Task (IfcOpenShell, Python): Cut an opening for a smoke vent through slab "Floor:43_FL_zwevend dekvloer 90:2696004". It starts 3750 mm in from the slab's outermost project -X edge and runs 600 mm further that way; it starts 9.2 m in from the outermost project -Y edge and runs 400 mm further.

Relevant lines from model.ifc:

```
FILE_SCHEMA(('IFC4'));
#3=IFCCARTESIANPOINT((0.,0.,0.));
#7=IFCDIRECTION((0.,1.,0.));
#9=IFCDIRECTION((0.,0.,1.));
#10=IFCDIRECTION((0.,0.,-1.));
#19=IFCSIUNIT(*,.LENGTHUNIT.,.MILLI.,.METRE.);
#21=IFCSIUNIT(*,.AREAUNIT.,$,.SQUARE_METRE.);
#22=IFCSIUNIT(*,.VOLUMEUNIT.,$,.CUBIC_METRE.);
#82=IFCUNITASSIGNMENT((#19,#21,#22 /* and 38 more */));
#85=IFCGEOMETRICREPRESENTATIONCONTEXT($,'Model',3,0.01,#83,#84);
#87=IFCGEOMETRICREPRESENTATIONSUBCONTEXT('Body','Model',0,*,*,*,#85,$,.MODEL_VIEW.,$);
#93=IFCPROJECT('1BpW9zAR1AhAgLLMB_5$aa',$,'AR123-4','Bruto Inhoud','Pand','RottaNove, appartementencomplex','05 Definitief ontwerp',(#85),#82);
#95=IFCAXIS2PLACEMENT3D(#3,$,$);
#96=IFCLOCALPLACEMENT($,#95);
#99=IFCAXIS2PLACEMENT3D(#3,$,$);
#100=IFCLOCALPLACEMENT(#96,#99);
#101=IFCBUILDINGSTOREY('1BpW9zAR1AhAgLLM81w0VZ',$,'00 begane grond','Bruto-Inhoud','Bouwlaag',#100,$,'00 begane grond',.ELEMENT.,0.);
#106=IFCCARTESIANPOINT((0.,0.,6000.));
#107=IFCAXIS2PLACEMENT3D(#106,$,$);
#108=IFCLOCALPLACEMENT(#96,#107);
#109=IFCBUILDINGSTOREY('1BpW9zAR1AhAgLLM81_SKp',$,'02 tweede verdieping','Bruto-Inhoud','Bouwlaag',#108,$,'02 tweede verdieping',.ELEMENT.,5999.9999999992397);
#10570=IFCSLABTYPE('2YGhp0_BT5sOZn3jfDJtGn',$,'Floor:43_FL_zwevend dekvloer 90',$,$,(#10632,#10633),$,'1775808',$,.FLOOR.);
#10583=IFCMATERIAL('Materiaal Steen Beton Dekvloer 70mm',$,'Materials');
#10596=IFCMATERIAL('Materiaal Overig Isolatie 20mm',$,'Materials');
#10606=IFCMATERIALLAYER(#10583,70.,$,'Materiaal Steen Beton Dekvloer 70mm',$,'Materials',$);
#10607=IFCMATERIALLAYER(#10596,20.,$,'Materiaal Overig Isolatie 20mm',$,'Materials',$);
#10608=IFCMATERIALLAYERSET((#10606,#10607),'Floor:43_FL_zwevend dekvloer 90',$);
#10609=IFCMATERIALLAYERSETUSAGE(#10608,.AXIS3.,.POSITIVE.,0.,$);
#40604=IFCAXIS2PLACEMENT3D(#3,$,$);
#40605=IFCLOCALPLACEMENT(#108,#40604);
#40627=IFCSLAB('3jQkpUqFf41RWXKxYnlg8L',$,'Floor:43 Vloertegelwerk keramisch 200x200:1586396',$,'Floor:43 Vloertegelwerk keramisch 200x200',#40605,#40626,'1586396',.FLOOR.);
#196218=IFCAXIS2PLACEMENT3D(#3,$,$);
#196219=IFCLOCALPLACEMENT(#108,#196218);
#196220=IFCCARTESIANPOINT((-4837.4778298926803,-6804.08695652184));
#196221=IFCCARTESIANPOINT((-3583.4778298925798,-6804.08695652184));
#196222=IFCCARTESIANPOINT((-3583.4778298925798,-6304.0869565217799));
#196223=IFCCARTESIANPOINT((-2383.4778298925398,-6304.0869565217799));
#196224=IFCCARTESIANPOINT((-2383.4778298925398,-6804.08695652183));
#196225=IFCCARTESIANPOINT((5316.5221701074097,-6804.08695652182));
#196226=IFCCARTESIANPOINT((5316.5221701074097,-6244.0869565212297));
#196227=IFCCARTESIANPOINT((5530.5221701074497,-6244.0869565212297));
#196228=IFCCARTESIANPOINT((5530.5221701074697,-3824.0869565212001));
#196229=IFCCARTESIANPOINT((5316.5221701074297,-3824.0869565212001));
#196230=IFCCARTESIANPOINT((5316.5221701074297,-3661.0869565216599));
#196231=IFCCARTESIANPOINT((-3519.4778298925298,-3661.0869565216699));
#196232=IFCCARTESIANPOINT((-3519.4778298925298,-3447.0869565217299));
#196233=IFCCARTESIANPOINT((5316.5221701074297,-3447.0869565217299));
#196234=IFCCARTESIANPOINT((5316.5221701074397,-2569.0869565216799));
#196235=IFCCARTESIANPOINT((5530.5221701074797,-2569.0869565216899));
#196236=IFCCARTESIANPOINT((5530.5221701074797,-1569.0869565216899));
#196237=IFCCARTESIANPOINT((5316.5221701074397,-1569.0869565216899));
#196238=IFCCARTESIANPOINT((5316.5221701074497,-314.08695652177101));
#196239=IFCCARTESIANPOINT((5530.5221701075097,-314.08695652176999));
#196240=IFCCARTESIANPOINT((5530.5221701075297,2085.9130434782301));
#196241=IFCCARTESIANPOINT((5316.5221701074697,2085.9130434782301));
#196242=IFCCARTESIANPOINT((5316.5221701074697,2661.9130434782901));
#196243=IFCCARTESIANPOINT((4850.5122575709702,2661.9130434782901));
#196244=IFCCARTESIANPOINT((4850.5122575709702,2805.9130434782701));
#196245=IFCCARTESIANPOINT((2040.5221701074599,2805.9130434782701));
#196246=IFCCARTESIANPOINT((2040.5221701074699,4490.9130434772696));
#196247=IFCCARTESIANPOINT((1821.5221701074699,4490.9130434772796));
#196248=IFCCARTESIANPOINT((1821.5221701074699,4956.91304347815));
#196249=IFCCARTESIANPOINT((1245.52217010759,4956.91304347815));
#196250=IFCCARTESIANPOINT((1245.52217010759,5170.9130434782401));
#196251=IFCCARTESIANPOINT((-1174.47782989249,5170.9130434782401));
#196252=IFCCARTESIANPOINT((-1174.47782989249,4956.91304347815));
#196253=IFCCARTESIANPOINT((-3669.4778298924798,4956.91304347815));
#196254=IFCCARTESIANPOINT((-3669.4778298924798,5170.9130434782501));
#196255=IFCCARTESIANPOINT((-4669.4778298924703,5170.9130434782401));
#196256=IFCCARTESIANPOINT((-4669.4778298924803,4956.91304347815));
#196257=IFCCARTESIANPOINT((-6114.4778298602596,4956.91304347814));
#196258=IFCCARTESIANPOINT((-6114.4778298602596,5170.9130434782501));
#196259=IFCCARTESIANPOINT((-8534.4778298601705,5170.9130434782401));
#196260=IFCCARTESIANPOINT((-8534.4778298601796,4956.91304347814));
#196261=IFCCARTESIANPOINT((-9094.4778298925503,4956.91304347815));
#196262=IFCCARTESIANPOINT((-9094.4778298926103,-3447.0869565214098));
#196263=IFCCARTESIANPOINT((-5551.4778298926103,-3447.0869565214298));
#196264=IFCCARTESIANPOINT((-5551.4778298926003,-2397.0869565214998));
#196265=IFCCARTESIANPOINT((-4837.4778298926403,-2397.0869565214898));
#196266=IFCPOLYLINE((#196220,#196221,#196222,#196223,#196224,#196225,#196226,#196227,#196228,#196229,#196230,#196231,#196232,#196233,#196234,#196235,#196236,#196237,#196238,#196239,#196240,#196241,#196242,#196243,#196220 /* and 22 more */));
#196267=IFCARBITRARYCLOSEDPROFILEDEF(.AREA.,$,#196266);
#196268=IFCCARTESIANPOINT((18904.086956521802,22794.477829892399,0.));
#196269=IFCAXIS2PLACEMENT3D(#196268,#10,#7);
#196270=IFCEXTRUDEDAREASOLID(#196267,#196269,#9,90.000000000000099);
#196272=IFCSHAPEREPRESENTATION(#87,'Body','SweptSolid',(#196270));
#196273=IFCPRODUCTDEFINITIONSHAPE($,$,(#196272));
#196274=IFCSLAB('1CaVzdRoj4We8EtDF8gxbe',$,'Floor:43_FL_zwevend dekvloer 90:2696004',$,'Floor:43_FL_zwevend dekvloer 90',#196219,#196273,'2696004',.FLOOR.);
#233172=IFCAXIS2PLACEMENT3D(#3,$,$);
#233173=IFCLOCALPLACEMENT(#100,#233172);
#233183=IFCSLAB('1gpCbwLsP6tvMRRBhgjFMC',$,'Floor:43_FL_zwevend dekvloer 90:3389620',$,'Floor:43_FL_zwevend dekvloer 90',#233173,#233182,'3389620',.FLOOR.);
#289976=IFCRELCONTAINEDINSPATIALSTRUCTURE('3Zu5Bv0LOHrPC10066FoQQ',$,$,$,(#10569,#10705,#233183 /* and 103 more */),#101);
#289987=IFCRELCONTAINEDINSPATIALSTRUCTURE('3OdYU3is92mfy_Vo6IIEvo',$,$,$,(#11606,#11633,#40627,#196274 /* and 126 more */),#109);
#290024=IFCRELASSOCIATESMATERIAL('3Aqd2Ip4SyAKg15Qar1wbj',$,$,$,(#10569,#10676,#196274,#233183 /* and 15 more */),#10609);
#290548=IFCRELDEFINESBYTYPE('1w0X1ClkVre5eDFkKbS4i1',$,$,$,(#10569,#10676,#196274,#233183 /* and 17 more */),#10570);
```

```python
import numpy as np
import ifcopenshell
import ifcopenshell.api.feature
import ifcopenshell.api.geometry
import ifcopenshell.api.root
import ifcopenshell.geom
import ifcopenshell.util.placement
import ifcopenshell.util.representation
import ifcopenshell.util.shape
import ifcopenshell.util.unit

model = ifcopenshell.open("model.ifc")
unit_scale = ifcopenshell.util.unit.calculate_unit_scale(model)
settings = ifcopenshell.geom.settings()


def volume(element):
    """Net volume in cubic metres, openings subtracted."""
    shape = ifcopenshell.geom.create_shape(settings, element)
    return ifcopenshell.util.shape.get_volume(shape.geometry)


slab = model.by_guid("1CaVzdRoj4We8EtDF8gxbe")
before = volume(slab)

# Extent in the slab's own axes, in metres. The edges named are its -X and -Y sides.
slab_shape = ifcopenshell.geom.create_shape(settings, slab)
vertices = ifcopenshell.util.shape.get_vertices(slab_shape.geometry)
x_min, y_min, bottom = vertices.min(axis=0)
top = vertices[:, 2].max()

opening = ifcopenshell.api.root.create_entity(model, ifc_class="IfcOpeningElement", name="Smoke vent opening", predefined_type="OPENING")
context = ifcopenshell.util.representation.get_context(model, "Model", "Body", "MODEL_VIEW")
width, depth = 0.6, 0.4
outline = [(0.0, 0.0), (width, 0.0), (width, depth), (0.0, depth), (0.0, 0.0)]
# Overshoot both faces by 50 mm so the cut is clean.
shape = ifcopenshell.api.geometry.add_slab_representation(
    model, context=context, depth=top - bottom + 0.1, polyline=outline
)
ifcopenshell.api.geometry.assign_representation(model, product=opening, representation=shape)

matrix = ifcopenshell.util.placement.get_local_placement(slab.ObjectPlacement)
matrix[:, 3] = matrix @ np.append(np.array([x_min + 3.75, y_min + 9.2, bottom - 0.05]) / unit_scale, 1.0)
ifcopenshell.api.geometry.edit_object_placement(model, product=opening, matrix=matrix, is_si=False)
ifcopenshell.api.feature.add_feature(model, feature=opening, element=slab)

after = volume(slab)

print(f"slab volume {before:.3f} -> {after:.3f} m3")

model.write("model_updated.ifc")
```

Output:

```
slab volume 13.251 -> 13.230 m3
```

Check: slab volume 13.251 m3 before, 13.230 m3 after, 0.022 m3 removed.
